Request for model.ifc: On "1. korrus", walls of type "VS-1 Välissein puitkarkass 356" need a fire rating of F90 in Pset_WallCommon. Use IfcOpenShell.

First a look at what the model holds.

```python
import ifcopenshell
import ifcopenshell.util.element

model = ifcopenshell.open("model.ifc")
print(model.schema)
storey = next(s for s in model.by_type("IfcBuildingStorey") if s.Name == "1. korrus")
walls = [e for e in ifcopenshell.util.element.get_decomposition(storey) if e.is_a("IfcWall")]
seen = {}
for e in walls:
    element_type = ifcopenshell.util.element.get_type(e)
    key = (element_type.Name if element_type != e and element_type else None, ifcopenshell.util.element.get_pset(e, "Pset_WallCommon", "FireRating"))
    seen[key] = seen.get(key, 0) + 1
for (name, value), count in sorted(seen.items(), key=str):
    print(count, "x", name, "|", value)
```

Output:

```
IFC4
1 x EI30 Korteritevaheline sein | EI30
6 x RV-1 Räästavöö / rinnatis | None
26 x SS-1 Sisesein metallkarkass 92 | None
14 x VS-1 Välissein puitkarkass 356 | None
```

```python
import ifcopenshell
import ifcopenshell.api.pset
import ifcopenshell.util.element

model = ifcopenshell.open("model.ifc")

storey = next(s for s in model.by_type("IfcBuildingStorey") if s.Name == "1. korrus")
walls = [e for e in ifcopenshell.util.element.get_decomposition(storey) if e.is_a("IfcWall")]

count = 0
for e in walls:
    element_type = ifcopenshell.util.element.get_type(e)
    if element_type in (None, e) or element_type.Name != "VS-1 Välissein puitkarkass 356":
        continue
    # add_pset returns the element's existing set when there is one.
    pset = ifcopenshell.api.pset.add_pset(model, product=e, name="Pset_WallCommon")
    ifcopenshell.api.pset.edit_pset(model, pset=pset, properties={"FireRating": "F90"})
    count += 1

print(count, "walls updated")

model.write("model_v2.ifc")
```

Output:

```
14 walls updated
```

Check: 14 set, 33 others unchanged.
